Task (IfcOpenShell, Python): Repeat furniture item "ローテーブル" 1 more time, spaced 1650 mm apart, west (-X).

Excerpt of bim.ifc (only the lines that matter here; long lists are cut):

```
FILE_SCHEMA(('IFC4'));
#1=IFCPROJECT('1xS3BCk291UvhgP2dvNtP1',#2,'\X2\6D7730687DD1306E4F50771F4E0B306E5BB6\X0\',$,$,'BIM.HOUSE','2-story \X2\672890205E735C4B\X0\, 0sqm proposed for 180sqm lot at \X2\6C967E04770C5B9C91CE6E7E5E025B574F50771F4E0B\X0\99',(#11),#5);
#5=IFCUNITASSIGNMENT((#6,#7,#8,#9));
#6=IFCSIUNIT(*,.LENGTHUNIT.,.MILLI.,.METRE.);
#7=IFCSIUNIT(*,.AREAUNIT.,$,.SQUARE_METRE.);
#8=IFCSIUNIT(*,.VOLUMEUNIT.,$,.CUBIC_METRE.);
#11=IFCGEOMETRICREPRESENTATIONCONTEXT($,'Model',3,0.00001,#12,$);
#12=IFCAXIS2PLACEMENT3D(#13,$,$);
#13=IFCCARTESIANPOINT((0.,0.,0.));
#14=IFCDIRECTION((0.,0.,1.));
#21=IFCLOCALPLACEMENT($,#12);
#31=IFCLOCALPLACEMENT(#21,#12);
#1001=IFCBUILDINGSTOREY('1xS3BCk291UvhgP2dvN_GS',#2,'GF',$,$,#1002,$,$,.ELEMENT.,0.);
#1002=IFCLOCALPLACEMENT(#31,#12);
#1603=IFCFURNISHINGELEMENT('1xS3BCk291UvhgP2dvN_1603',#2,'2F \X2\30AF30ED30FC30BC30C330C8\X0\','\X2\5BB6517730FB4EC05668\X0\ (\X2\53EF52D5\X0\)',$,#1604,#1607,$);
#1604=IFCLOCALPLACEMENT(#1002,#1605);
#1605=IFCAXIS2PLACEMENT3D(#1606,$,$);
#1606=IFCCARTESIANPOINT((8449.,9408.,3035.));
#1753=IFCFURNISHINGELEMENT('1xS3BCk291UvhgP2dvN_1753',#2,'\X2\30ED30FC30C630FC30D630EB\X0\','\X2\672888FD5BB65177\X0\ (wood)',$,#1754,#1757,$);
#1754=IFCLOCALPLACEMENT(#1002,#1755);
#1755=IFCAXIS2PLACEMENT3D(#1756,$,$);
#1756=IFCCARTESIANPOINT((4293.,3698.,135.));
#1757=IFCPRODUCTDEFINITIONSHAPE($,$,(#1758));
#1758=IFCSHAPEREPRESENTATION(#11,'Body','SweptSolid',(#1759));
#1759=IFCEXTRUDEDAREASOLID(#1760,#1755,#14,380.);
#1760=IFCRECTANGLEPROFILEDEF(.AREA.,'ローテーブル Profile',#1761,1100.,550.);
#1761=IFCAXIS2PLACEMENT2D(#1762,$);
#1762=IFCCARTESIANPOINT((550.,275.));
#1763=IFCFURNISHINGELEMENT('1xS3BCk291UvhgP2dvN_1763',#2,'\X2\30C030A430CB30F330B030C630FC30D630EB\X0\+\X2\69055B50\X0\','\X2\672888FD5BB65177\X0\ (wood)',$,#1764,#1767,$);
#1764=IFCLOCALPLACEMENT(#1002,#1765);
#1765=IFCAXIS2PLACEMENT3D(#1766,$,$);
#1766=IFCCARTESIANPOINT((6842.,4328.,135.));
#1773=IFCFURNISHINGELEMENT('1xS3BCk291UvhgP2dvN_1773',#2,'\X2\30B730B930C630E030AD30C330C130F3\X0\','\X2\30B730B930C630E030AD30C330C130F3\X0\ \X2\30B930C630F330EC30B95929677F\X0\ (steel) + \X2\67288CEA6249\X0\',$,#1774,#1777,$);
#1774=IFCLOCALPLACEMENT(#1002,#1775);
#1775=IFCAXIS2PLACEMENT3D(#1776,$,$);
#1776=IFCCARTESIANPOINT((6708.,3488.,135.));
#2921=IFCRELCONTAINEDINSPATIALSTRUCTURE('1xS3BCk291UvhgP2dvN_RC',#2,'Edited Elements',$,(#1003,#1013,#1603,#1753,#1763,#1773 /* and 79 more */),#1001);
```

```python
import numpy as np
import ifcopenshell
import ifcopenshell.api.geometry
import ifcopenshell.api.root
import ifcopenshell.util.element
import ifcopenshell.util.placement

model = ifcopenshell.open("bim.ifc")


def reuse_history(source, copy):
    """copy_class also copies each property set's owner history, people and application; keep the originals."""
    for rel in copy.IsDefinedBy:
        if rel.is_a("IfcRelDefinesByProperties") and (history := rel.RelatingPropertyDefinition.OwnerHistory):
            rel.RelatingPropertyDefinition.OwnerHistory = source.OwnerHistory
            ifcopenshell.util.element.remove_deep2(model, history)


source = model.by_id(1753)
base = ifcopenshell.util.placement.get_local_placement(source.ObjectPlacement)
step = np.array([-1.0, 0.0, 0.0]) * 1650.0

for i in range(1, 2):
    copy = ifcopenshell.api.root.copy_class(model, product=source)
    copy.Representation = ifcopenshell.util.element.copy_deep(
        model, source.Representation, exclude=["IfcGeometricRepresentationContext", "IfcRepresentationMap"]
    )
    reuse_history(source, copy)
    matrix = base.copy()
    matrix[:3, 3] += i * step
    print("added at", matrix[:3, 3].round(3) + 0.0)
    ifcopenshell.api.geometry.edit_object_placement(model, product=copy, matrix=matrix, is_si=False)

model.write("bim_v2.ifc")
```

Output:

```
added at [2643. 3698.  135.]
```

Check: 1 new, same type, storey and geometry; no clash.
